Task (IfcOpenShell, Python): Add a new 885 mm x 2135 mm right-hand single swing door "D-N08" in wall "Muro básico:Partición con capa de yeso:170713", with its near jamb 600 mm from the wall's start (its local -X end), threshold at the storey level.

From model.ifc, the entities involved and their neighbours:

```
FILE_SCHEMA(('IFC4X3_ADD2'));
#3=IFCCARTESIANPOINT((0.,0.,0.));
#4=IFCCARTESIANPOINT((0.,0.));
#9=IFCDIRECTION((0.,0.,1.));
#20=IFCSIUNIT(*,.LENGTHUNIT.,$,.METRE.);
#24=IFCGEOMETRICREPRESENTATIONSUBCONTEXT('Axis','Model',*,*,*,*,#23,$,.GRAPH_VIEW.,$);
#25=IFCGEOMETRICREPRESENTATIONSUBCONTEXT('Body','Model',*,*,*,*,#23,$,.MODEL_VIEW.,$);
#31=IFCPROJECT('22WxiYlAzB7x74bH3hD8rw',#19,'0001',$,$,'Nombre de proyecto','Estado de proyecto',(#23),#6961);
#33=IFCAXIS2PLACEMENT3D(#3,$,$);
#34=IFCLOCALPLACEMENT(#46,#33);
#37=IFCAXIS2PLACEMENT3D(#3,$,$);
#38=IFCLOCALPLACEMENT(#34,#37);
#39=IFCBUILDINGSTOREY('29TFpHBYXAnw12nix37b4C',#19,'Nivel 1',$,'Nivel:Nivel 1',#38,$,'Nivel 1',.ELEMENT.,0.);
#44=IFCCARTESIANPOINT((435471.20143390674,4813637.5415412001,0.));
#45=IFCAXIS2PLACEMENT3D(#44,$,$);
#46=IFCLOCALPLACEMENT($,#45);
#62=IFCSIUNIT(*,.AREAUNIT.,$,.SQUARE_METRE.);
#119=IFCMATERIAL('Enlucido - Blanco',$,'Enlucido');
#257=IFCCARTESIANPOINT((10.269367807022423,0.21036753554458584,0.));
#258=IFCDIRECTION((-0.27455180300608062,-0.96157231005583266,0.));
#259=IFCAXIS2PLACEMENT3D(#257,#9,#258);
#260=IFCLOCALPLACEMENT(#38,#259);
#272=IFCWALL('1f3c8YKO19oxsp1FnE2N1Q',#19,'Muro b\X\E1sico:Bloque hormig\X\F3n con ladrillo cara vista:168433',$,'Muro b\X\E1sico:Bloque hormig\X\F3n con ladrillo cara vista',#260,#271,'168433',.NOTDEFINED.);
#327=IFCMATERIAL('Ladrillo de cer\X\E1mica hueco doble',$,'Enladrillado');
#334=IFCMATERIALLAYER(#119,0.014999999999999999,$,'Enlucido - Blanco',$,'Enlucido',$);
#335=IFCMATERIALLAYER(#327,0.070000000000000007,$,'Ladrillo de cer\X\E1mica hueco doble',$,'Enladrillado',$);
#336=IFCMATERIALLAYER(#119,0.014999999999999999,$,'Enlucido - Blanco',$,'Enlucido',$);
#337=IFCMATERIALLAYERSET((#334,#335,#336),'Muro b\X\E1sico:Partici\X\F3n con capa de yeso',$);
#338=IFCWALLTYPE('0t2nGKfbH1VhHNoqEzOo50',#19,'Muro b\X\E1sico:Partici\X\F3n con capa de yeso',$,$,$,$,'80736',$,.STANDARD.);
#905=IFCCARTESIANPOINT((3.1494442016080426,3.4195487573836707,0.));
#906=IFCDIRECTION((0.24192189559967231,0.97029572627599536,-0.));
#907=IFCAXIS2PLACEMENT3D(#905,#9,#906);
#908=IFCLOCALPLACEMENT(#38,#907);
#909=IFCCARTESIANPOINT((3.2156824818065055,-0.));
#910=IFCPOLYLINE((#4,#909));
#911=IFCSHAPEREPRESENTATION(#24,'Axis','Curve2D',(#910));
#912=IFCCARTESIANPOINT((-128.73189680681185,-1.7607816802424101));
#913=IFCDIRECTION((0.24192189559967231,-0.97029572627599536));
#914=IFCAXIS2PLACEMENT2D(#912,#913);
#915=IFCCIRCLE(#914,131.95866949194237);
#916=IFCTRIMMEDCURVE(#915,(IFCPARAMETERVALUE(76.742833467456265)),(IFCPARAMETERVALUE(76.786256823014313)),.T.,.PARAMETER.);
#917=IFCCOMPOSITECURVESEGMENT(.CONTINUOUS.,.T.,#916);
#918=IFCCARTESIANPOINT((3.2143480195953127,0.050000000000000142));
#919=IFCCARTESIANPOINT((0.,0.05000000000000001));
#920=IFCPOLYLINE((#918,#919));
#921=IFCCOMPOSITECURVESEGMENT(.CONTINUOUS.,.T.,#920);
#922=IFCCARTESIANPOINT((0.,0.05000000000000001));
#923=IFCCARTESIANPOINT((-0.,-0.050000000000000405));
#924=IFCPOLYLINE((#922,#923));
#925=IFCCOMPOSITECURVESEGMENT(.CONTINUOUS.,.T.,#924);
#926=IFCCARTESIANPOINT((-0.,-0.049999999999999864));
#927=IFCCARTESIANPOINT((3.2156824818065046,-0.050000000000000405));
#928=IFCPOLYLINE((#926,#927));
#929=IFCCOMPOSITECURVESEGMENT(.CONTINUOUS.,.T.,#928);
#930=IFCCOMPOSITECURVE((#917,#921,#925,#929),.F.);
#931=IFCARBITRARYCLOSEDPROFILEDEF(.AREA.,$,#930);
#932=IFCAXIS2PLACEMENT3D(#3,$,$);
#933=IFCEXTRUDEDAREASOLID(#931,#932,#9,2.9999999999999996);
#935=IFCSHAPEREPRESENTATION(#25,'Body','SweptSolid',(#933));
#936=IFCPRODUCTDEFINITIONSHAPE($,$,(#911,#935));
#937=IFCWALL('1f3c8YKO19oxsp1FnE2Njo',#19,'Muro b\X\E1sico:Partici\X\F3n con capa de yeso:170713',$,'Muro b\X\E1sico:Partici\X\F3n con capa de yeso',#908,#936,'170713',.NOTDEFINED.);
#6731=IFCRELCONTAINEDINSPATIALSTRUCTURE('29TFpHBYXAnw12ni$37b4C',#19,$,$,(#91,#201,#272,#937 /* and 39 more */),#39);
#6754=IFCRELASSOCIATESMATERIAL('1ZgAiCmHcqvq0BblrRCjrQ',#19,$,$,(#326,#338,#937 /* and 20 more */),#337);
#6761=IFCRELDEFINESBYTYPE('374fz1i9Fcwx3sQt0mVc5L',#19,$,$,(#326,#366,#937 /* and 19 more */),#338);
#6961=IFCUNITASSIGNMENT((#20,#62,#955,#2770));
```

```python
import numpy as np
import ifcopenshell
import ifcopenshell.api.feature
import ifcopenshell.api.geometry
import ifcopenshell.api.root
import ifcopenshell.api.spatial
import ifcopenshell.geom
import ifcopenshell.util.element
import ifcopenshell.util.placement
import ifcopenshell.util.representation
import ifcopenshell.util.shape
import ifcopenshell.util.unit

model = ifcopenshell.open("model.ifc")
unit_scale = ifcopenshell.util.unit.calculate_unit_scale(model)
settings = ifcopenshell.geom.settings()


def volume(element):
    """Net volume in cubic metres, openings subtracted."""
    shape = ifcopenshell.geom.create_shape(settings, element)
    return ifcopenshell.util.shape.get_volume(shape.geometry)


wall = model.by_id(937)
storey = ifcopenshell.util.element.get_container(wall, ifc_class="IfcBuildingStorey")
context = ifcopenshell.util.representation.get_context(model, "Model", "Body", "MODEL_VIEW")
before = volume(wall)

width, height, from_end, sill = 0.885, 2.135, 0.6, 0.0  # metres

# The wall runs along its own X axis, and the end named is its -X end.
wall_shape = ifcopenshell.geom.create_shape(settings, wall)
x, y, z = ifcopenshell.util.shape.get_vertices(wall_shape.geometry).T
start = x.min() + from_end
face, thickness = float(y.min()), float(y.max() - y.min())
wall_matrix = ifcopenshell.util.placement.get_local_placement(wall.ObjectPlacement)
level = ifcopenshell.util.placement.get_local_placement(storey.ObjectPlacement)[2, 3]


def in_wall(x, y):
    """Placement at x, y metres in the wall's axes, at sill height."""
    matrix = wall_matrix.copy()
    matrix[:, 3] = wall_matrix @ np.array([x / unit_scale, y / unit_scale, 0.0, 1.0])
    matrix[2, 3] = level + sill / unit_scale
    return matrix


# Opening: a box that overshoots both wall faces by 50 mm.
opening = ifcopenshell.api.root.create_entity(model, ifc_class="IfcOpeningElement", predefined_type="OPENING")
box = ifcopenshell.api.geometry.add_wall_representation(
    model, context=context, length=width, height=height, thickness=thickness + 0.1
)
ifcopenshell.api.geometry.assign_representation(model, product=opening, representation=box)
ifcopenshell.api.geometry.edit_object_placement(model, product=opening, matrix=in_wall(start, face - 0.05), is_si=False)
ifcopenshell.api.feature.add_feature(model, feature=opening, element=wall)

door = ifcopenshell.api.root.create_entity(model, ifc_class="IfcDoor", name="D-N08", predefined_type="DOOR")
door.OverallWidth, door.OverallHeight = width / unit_scale, height / unit_scale
door.OperationType = "SINGLE_SWING_RIGHT"
body = ifcopenshell.api.geometry.add_door_representation(
    model,
    context=context,
    overall_width=door.OverallWidth,
    overall_height=door.OverallHeight,
    operation_type="SINGLE_SWING_RIGHT",
    lining_properties={"LiningDepth": thickness / unit_scale, "ThresholdDepth": thickness / unit_scale},
)
ifcopenshell.api.geometry.assign_representation(model, product=door, representation=body)
ifcopenshell.api.spatial.assign_container(model, products=[door], relating_structure=storey)
ifcopenshell.api.feature.add_filling(model, opening=opening, element=door)

# The lining spans the wall, so the door starts at the wall face.
ifcopenshell.api.geometry.edit_object_placement(model, product=door, matrix=in_wall(start, face), is_si=False)

after = volume(wall)

print(f"wall volume {before:.3f} -> {after:.3f} m3")

model.write("model_edited.ifc")
```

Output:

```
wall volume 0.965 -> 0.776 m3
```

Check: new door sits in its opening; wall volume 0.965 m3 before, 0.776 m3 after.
